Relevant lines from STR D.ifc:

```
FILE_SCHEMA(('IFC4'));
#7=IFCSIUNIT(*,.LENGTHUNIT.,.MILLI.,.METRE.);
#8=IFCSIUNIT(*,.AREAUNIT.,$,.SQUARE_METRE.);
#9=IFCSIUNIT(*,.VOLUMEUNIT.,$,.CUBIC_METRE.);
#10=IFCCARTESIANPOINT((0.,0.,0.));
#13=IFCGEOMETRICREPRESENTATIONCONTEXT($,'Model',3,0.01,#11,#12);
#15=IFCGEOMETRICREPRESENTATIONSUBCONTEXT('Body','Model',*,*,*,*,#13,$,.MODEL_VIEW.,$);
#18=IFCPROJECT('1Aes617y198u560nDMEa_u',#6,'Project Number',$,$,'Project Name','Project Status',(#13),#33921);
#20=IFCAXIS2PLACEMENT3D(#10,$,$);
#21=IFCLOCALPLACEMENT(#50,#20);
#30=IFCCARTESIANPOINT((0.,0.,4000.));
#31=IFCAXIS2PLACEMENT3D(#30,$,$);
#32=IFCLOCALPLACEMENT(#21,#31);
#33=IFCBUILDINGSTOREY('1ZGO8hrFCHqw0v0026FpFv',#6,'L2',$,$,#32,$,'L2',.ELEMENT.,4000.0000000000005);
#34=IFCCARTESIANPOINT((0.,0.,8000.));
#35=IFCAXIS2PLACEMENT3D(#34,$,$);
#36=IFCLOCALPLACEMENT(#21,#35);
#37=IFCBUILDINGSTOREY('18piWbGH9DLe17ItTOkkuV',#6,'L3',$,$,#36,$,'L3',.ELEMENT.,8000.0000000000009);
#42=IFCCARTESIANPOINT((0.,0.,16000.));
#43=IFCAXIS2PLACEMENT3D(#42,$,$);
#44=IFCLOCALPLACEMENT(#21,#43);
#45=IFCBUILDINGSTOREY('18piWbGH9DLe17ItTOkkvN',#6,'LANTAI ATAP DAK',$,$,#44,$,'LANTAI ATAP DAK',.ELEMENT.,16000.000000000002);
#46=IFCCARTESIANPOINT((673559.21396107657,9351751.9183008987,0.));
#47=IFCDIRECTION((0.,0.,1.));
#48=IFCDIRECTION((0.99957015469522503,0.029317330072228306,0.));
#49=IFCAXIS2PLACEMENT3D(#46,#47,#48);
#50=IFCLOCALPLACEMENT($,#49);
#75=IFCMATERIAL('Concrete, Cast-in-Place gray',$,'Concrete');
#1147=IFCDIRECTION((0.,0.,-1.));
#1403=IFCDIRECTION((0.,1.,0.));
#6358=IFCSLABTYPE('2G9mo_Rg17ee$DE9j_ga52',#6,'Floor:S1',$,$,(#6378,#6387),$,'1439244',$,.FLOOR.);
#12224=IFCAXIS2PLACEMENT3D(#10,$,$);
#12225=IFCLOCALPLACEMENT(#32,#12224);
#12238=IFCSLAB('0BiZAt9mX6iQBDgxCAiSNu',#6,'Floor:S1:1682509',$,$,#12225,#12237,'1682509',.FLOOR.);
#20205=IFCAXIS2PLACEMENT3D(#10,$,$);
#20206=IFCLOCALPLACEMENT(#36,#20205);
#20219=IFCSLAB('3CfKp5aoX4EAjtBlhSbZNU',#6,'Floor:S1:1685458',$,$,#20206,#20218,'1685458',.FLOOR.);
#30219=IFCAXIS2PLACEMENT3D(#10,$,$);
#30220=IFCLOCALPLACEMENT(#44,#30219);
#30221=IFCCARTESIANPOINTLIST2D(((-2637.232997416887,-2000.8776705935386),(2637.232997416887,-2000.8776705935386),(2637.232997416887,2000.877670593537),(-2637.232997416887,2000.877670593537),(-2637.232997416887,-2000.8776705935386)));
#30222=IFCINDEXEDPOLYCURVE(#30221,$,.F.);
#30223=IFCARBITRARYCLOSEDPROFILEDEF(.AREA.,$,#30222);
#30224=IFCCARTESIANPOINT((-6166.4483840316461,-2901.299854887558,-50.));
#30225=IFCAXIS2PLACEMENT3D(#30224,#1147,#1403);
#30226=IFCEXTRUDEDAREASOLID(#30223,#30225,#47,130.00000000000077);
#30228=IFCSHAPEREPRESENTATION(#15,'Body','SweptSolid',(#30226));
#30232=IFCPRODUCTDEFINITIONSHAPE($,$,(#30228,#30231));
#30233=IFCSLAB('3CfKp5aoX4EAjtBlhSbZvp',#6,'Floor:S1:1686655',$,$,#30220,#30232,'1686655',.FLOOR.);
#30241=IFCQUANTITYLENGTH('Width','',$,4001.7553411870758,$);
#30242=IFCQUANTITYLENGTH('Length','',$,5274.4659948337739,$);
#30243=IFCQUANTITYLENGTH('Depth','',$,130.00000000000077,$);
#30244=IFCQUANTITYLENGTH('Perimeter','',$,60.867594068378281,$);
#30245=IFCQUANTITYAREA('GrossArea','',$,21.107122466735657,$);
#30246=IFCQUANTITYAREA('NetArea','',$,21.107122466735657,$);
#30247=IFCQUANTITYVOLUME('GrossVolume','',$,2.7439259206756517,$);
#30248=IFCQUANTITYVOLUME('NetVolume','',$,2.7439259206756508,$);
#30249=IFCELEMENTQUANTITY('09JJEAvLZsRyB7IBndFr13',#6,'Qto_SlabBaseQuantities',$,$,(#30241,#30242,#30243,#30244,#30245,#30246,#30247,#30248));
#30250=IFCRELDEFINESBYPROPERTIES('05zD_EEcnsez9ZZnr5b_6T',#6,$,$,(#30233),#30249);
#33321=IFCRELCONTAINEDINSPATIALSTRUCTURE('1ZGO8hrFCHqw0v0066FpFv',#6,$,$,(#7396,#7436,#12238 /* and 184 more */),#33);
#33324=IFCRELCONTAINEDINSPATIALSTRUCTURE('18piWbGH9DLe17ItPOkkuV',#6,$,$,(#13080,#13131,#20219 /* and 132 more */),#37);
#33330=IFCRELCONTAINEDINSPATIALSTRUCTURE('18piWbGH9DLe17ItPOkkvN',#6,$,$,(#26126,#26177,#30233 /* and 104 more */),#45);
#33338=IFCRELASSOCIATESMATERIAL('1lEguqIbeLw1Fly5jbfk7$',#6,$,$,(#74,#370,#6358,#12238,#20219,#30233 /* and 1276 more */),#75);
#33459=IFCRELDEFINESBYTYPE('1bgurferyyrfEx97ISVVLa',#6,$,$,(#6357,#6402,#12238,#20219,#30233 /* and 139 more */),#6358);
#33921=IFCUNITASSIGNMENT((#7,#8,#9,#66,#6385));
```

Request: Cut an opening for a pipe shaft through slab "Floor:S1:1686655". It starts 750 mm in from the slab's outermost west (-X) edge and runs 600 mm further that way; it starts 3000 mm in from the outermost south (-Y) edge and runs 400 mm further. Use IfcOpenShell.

```python
import numpy as np
import ifcopenshell
import ifcopenshell.api.feature
import ifcopenshell.api.geometry
import ifcopenshell.api.pset
import ifcopenshell.api.root
import ifcopenshell.geom
import ifcopenshell.util.element
import ifcopenshell.util.placement
import ifcopenshell.util.representation
import ifcopenshell.util.shape
import ifcopenshell.util.unit

model = ifcopenshell.open("STR D.ifc")
unit_scale = ifcopenshell.util.unit.calculate_unit_scale(model)
area_scale = ifcopenshell.util.unit.calculate_unit_scale(model, "AREAUNIT")
volume_scale = ifcopenshell.util.unit.calculate_unit_scale(model, "VOLUMEUNIT")
settings = ifcopenshell.geom.settings()


def volume(element):
    """Net volume in cubic metres, openings subtracted."""
    shape = ifcopenshell.geom.create_shape(settings, element)
    return ifcopenshell.util.shape.get_volume(shape.geometry)


slab = model.by_guid("3CfKp5aoX4EAjtBlhSbZvp")
before = volume(slab)

# Extent in the slab's own axes, in metres. The edges named are its -X and -Y sides.
slab_shape = ifcopenshell.geom.create_shape(settings, slab)
vertices = ifcopenshell.util.shape.get_vertices(slab_shape.geometry)
x_min, y_min, bottom = vertices.min(axis=0)
top = vertices[:, 2].max()

opening = ifcopenshell.api.root.create_entity(model, ifc_class="IfcOpeningElement", name="Pipe shaft opening", predefined_type="OPENING")
context = ifcopenshell.util.representation.get_context(model, "Model", "Body", "MODEL_VIEW")
width, depth = 0.6, 0.4
outline = [(0.0, 0.0), (width, 0.0), (width, depth), (0.0, depth), (0.0, 0.0)]
# Overshoot both faces by 50 mm so the cut is clean.
shape = ifcopenshell.api.geometry.add_slab_representation(
    model, context=context, depth=top - bottom + 0.1, polyline=outline
)
ifcopenshell.api.geometry.assign_representation(model, product=opening, representation=shape)

matrix = ifcopenshell.util.placement.get_local_placement(slab.ObjectPlacement)
matrix[:, 3] = matrix @ np.append(np.array([x_min + 0.75, y_min + 3, bottom - 0.05]) / unit_scale, 1.0)
ifcopenshell.api.geometry.edit_object_placement(model, product=opening, matrix=matrix, is_si=False)
ifcopenshell.api.feature.add_feature(model, feature=opening, element=slab)

after = volume(slab)

# Update the slab's stored quantities.
qto = model.by_id(ifcopenshell.util.element.get_pset(slab, "Qto_SlabBaseQuantities", should_inherit=False)["id"])
ifcopenshell.api.pset.edit_qto(model, qto=qto, properties={
    "NetArea": after / (top - bottom) / area_scale,
    "NetVolume": after / volume_scale,
})

print(f"slab volume {before:.3f} -> {after:.3f} m3")

model.write("STR D_rev.ifc")
```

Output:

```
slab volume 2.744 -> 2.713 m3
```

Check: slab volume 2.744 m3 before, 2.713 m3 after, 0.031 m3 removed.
